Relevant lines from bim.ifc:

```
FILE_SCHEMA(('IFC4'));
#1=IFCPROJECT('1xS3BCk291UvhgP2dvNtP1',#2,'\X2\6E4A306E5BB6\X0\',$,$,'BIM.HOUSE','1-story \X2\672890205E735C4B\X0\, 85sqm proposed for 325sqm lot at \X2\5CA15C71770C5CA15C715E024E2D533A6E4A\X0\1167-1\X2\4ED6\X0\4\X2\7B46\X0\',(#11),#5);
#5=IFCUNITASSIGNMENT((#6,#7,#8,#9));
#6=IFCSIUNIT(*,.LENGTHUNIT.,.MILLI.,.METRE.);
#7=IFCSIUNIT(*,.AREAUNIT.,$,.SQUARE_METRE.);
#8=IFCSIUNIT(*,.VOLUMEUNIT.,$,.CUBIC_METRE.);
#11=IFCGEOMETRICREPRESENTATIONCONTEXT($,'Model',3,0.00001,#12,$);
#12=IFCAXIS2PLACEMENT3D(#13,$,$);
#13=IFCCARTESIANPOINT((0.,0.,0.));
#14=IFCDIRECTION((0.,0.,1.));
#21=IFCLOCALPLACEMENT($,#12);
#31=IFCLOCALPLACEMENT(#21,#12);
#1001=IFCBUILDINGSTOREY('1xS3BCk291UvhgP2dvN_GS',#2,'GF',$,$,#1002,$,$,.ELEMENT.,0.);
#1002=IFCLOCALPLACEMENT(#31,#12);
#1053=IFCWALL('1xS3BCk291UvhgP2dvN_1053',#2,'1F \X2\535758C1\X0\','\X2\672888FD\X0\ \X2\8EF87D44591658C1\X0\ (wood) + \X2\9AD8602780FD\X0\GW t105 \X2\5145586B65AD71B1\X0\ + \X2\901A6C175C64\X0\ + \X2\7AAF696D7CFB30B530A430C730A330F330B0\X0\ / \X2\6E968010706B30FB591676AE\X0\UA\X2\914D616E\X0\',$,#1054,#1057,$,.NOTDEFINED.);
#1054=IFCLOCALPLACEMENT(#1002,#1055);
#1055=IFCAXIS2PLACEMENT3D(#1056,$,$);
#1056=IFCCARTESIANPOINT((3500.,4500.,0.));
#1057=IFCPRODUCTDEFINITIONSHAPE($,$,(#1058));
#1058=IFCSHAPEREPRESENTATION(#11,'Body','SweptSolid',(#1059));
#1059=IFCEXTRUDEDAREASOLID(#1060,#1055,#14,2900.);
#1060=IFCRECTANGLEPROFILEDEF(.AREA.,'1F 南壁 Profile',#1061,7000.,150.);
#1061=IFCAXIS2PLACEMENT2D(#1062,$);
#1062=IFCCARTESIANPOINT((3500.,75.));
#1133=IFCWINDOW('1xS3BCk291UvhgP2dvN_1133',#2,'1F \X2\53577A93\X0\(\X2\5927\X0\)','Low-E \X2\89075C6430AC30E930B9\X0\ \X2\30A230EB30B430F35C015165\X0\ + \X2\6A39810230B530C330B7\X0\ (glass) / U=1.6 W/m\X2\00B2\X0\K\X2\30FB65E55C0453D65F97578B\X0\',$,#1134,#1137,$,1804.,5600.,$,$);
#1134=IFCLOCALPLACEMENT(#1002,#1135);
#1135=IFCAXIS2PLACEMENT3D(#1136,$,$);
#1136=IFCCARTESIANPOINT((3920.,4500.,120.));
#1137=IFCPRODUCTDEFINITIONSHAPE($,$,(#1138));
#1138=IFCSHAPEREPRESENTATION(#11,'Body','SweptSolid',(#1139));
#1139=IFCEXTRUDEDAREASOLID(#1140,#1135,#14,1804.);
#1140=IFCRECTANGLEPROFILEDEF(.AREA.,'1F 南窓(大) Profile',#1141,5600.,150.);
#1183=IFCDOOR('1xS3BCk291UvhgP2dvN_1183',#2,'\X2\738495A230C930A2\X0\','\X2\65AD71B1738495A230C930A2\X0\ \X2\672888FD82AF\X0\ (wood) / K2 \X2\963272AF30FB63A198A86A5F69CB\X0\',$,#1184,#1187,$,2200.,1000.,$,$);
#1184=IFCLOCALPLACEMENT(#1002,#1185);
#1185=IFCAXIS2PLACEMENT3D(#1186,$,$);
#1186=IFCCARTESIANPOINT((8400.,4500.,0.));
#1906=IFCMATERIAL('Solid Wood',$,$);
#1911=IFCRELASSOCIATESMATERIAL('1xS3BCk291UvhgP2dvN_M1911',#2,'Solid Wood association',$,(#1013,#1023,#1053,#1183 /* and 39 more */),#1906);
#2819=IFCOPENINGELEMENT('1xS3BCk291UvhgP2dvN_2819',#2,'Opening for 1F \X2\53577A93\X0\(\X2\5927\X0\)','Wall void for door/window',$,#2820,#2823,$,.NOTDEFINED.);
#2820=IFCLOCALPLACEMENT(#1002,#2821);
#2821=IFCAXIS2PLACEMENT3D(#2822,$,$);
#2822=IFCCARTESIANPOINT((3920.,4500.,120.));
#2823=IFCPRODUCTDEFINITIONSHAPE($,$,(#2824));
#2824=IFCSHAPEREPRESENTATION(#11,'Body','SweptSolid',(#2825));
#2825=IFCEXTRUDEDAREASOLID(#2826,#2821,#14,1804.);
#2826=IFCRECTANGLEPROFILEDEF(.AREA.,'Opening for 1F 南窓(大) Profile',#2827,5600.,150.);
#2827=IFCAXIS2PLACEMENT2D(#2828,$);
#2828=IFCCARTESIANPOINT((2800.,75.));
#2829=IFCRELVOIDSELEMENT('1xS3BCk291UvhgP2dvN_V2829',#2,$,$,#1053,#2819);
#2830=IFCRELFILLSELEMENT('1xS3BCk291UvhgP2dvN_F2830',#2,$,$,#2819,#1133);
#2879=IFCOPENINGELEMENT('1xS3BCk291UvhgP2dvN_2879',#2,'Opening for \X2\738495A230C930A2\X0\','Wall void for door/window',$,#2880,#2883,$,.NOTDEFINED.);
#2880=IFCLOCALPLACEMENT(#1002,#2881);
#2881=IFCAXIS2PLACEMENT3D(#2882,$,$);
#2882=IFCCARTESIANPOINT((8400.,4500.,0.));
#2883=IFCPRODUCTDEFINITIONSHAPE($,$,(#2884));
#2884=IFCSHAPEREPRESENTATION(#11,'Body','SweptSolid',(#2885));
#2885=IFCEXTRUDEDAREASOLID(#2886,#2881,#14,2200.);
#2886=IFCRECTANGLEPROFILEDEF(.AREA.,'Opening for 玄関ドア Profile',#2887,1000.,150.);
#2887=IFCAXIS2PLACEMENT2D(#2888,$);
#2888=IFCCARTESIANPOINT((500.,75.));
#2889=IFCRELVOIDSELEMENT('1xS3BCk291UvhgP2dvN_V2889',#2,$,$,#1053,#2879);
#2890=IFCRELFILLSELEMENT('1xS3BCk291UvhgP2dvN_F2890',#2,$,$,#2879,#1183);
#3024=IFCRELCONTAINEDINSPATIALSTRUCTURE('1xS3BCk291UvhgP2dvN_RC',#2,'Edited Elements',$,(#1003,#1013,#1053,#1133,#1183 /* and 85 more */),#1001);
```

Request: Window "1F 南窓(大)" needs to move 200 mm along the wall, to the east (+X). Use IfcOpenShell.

```python
import ifcopenshell
import ifcopenshell.api.geometry
import ifcopenshell.util.placement
import ifcopenshell.util.unit

model = ifcopenshell.open("bim.ifc")
unit_scale = ifcopenshell.util.unit.calculate_unit_scale(model)

window = model.by_id(1133)
opening = window.FillsVoids[0].RelatingOpeningElement
wall = opening.VoidsElements[0].RelatingBuildingElement

wall_matrix = ifcopenshell.util.placement.get_local_placement(wall.ObjectPlacement)
shift = wall_matrix[:3, 0] * 0.2 / unit_scale
before = ifcopenshell.util.placement.get_local_placement(window.ObjectPlacement)[:3, 3].copy()

# The window is not placed relative to its opening, so move both.
for product in (opening, window):
    matrix = ifcopenshell.util.placement.get_local_placement(product.ObjectPlacement)
    matrix[:3, 3] += shift
    ifcopenshell.api.geometry.edit_object_placement(model, product=product, matrix=matrix, is_si=False)

after = ifcopenshell.util.placement.get_local_placement(window.ObjectPlacement)[:3, 3]
print("window moved by", (after - before).round(3) + 0.0)

model.write("bim_rev.ifc")
```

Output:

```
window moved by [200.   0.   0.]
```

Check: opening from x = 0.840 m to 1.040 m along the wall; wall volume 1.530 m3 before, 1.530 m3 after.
